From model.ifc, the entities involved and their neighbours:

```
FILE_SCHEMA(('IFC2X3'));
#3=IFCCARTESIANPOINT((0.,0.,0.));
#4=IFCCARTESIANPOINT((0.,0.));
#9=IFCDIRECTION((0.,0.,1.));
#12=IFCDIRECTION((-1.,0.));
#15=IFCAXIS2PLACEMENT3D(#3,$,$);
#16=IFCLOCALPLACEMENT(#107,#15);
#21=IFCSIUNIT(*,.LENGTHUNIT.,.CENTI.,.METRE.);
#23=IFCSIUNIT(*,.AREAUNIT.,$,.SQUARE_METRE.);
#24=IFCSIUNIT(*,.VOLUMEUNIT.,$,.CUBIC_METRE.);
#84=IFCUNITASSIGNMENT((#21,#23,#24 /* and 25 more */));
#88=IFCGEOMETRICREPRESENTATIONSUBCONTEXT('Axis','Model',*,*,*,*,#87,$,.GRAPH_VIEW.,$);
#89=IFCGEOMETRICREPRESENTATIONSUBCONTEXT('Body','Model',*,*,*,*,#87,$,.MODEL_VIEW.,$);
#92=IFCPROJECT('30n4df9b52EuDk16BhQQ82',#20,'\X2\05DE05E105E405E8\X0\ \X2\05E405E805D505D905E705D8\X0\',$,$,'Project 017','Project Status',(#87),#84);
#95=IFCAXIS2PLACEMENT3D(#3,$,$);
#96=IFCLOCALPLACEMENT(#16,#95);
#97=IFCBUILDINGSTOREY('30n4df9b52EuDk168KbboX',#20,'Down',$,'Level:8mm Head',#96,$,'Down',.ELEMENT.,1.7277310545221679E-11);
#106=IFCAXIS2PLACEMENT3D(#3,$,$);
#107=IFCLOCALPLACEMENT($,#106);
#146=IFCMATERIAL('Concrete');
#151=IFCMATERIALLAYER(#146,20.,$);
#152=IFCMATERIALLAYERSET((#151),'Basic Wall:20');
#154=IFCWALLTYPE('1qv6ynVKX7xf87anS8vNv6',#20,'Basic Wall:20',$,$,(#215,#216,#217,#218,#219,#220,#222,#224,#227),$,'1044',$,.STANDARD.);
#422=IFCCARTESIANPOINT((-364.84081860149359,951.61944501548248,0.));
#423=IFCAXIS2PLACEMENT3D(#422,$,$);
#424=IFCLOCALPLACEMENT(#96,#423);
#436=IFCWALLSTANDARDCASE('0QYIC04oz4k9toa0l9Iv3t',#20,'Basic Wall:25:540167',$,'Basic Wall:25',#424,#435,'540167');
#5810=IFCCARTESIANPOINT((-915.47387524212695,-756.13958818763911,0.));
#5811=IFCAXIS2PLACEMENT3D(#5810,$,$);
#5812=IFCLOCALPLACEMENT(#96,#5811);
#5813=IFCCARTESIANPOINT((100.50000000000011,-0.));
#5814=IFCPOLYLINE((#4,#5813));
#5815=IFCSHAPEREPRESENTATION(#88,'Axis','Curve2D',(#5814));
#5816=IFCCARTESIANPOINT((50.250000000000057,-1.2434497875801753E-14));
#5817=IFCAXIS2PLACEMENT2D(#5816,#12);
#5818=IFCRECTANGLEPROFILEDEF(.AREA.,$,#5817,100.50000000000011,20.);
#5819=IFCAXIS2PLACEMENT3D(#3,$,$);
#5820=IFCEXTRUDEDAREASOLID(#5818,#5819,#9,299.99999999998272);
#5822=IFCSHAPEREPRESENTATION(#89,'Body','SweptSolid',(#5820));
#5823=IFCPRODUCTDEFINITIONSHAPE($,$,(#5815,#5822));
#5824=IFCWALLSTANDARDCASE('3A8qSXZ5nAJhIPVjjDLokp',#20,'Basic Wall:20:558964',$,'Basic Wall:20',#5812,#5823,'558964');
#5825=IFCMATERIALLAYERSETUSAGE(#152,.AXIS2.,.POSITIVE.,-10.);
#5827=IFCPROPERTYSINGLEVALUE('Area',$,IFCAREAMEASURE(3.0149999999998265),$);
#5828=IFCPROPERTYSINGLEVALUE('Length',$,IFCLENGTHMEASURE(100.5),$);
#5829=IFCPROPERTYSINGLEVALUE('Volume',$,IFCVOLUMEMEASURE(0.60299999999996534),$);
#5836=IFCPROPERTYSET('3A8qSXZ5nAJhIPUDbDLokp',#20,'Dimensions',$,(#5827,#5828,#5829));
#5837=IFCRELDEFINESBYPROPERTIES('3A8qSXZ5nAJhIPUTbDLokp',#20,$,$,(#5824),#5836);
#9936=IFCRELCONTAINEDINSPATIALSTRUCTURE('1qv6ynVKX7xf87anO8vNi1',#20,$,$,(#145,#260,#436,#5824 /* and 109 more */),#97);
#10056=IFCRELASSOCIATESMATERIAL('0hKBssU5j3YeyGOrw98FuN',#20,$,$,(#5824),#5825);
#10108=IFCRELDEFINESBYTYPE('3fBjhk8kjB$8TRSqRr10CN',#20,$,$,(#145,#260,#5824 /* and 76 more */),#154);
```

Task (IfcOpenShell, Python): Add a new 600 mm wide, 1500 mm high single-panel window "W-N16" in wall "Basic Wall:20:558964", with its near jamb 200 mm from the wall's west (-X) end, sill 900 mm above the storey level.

```python
import numpy as np
import ifcopenshell
import ifcopenshell.api.feature
import ifcopenshell.api.geometry
import ifcopenshell.api.pset
import ifcopenshell.api.root
import ifcopenshell.api.spatial
import ifcopenshell.api.type
import ifcopenshell.geom
import ifcopenshell.util.element
import ifcopenshell.util.placement
import ifcopenshell.util.representation
import ifcopenshell.util.shape
import ifcopenshell.util.unit

model = ifcopenshell.open("model.ifc")
unit_scale = ifcopenshell.util.unit.calculate_unit_scale(model)
area_scale = ifcopenshell.util.unit.calculate_unit_scale(model, "AREAUNIT")
volume_scale = ifcopenshell.util.unit.calculate_unit_scale(model, "VOLUMEUNIT")
settings = ifcopenshell.geom.settings()


def volume(element):
    """Net volume in cubic metres, openings subtracted."""
    shape = ifcopenshell.geom.create_shape(settings, element)
    return ifcopenshell.util.shape.get_volume(shape.geometry)


wall = model.by_guid("3A8qSXZ5nAJhIPVjjDLokp")
storey = ifcopenshell.util.element.get_container(wall, ifc_class="IfcBuildingStorey")
context = ifcopenshell.util.representation.get_context(model, "Model", "Body", "MODEL_VIEW")
before = volume(wall)

width, height, from_end, sill = 0.6, 1.5, 0.2, 0.9  # metres

# The wall runs along its own X axis, and the end named is its -X end.
wall_shape = ifcopenshell.geom.create_shape(settings, wall)
x, y, z = ifcopenshell.util.shape.get_vertices(wall_shape.geometry).T
start = x.min() + from_end
face, thickness = float(y.min()), float(y.max() - y.min())
wall_matrix = ifcopenshell.util.placement.get_local_placement(wall.ObjectPlacement)
level = ifcopenshell.util.placement.get_local_placement(storey.ObjectPlacement)[2, 3]


def in_wall(x, y):
    """Placement at x, y metres in the wall's axes, at sill height."""
    matrix = wall_matrix.copy()
    matrix[:, 3] = wall_matrix @ np.array([x / unit_scale, y / unit_scale, 0.0, 1.0])
    matrix[2, 3] = level + sill / unit_scale
    return matrix


# Opening: a box that overshoots both wall faces by 50 mm.
opening = ifcopenshell.api.root.create_entity(model, ifc_class="IfcOpeningElement")
box = ifcopenshell.api.geometry.add_wall_representation(
    model, context=context, length=width, height=height, thickness=thickness + 0.1
)
ifcopenshell.api.geometry.assign_representation(model, product=opening, representation=box)
ifcopenshell.api.geometry.edit_object_placement(model, product=opening, matrix=in_wall(start, face - 0.05), is_si=False)
ifcopenshell.api.feature.add_feature(model, feature=opening, element=wall)

window = ifcopenshell.api.root.create_entity(model, ifc_class="IfcWindow", name="W-N16")
window.OverallWidth, window.OverallHeight = width / unit_scale, height / unit_scale
body = ifcopenshell.api.geometry.add_window_representation(
    model,
    context=context,
    overall_width=window.OverallWidth,
    overall_height=window.OverallHeight,
    partition_type="SINGLE_PANEL",
)
ifcopenshell.api.geometry.assign_representation(model, product=window, representation=body)
ifcopenshell.api.spatial.assign_container(model, products=[window], relating_structure=storey)
fills = ifcopenshell.api.feature.add_filling(model, opening=opening, element=window)
fills.OwnerHistory = window.OwnerHistory  # required in IFC2X3

# IFC2X3 keeps the operation on the window style.
style = ifcopenshell.api.root.create_entity(model, ifc_class="IfcWindowStyle", name="W-N16")
style.OperationType, style.ConstructionType = "SINGLE_PANEL", "NOTDEFINED"
style.ParameterTakesPrecedence = style.Sizeable = False
ifcopenshell.api.type.assign_type(model, related_objects=[window], relating_type=style)

# Centre the window in the wall's thickness.
ifcopenshell.api.geometry.edit_object_placement(model, product=window, matrix=in_wall(start, face), is_si=False)
window_shape = ifcopenshell.geom.create_shape(settings, window)
depth = ifcopenshell.util.shape.get_vertices(window_shape.geometry)[:, 1]
offset = face + thickness / 2 - (depth.min() + depth.max()) / 2
ifcopenshell.api.geometry.edit_object_placement(model, product=window, matrix=in_wall(start, offset), is_si=False)

after = volume(wall)

# Update the wall's stored quantities.
pset = model.by_id(ifcopenshell.util.element.get_pset(wall, "Dimensions", should_inherit=False)["id"])
ifcopenshell.api.pset.edit_pset(model, pset=pset, properties={
    "Area": model.create_entity("IfcAreaMeasure", after / thickness / area_scale),
    "Volume": model.create_entity("IfcVolumeMeasure", after / volume_scale),
})

print(f"wall volume {before:.3f} -> {after:.3f} m3")

model.write("model_updated.ifc")
```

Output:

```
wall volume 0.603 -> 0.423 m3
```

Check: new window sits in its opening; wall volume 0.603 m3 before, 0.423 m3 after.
